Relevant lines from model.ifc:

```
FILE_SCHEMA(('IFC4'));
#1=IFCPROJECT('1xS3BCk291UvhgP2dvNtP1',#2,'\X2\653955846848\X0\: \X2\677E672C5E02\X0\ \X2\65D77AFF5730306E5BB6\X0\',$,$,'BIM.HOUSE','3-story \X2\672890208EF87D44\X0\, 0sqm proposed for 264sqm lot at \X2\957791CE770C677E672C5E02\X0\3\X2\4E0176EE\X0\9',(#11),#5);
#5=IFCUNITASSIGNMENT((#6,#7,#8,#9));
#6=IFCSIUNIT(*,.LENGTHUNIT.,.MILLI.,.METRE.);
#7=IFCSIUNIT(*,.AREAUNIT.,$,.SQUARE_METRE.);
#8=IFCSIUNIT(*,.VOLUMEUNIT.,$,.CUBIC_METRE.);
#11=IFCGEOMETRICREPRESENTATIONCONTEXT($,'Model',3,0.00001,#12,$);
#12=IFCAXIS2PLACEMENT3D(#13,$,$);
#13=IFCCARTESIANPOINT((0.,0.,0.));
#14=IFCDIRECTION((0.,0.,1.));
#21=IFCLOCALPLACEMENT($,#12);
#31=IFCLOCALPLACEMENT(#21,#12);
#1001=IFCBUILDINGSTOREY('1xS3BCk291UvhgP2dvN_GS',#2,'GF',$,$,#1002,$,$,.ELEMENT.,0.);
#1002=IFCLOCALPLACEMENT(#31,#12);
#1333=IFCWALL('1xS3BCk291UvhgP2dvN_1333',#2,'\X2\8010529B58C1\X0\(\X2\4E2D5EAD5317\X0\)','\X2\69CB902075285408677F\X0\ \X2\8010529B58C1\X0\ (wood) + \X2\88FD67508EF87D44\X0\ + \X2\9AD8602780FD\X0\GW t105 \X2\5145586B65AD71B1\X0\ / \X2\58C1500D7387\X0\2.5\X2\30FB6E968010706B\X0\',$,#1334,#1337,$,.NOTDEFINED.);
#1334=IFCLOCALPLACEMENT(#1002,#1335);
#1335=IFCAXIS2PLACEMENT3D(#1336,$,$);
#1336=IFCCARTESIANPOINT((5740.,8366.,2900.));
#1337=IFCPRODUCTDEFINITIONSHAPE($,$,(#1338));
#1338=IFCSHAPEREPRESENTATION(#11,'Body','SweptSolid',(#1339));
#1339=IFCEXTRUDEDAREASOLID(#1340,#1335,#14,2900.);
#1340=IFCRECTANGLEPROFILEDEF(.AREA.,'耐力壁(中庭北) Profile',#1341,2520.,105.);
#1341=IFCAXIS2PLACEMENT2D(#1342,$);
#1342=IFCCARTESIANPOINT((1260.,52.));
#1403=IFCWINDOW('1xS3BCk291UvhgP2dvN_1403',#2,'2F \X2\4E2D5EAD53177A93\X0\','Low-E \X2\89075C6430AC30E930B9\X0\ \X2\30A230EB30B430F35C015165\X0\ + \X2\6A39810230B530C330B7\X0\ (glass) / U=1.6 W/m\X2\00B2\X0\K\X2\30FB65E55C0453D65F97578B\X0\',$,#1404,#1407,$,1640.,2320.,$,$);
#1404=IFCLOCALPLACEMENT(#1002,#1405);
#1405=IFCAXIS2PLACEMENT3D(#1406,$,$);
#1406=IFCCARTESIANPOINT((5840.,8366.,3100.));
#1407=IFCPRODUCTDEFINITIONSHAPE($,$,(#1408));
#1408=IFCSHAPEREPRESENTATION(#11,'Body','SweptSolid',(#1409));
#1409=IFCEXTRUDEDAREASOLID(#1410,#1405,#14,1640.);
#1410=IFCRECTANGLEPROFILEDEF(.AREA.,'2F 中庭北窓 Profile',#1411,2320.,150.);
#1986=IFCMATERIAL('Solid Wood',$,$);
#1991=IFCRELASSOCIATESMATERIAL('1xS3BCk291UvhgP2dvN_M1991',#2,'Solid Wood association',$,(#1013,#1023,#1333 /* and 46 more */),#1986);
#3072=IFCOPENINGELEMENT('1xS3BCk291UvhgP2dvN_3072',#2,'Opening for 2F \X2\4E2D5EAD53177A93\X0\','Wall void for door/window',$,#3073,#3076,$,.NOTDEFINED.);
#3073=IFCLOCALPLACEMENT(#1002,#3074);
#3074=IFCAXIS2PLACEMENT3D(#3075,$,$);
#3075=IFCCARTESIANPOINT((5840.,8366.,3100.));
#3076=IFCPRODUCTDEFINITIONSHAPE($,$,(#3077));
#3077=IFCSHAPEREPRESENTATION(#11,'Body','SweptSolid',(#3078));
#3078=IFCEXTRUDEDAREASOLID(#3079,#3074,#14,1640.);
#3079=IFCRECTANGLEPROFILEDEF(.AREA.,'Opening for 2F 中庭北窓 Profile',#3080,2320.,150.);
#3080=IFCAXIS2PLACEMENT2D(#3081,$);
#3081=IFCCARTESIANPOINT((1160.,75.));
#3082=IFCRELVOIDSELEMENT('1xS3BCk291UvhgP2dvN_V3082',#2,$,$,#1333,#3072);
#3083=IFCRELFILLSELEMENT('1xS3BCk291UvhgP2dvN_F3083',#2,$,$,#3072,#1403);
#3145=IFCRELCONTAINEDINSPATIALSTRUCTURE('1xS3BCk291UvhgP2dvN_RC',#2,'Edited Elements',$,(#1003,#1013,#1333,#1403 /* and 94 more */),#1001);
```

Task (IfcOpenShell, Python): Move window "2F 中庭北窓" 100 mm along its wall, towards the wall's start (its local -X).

```python
import ifcopenshell
import ifcopenshell.api.geometry
import ifcopenshell.util.placement
import ifcopenshell.util.unit

model = ifcopenshell.open("model.ifc")
unit_scale = ifcopenshell.util.unit.calculate_unit_scale(model)

window = model.by_id(1403)
opening = window.FillsVoids[0].RelatingOpeningElement
wall = opening.VoidsElements[0].RelatingBuildingElement

wall_matrix = ifcopenshell.util.placement.get_local_placement(wall.ObjectPlacement)
shift = wall_matrix[:3, 0] * -0.1 / unit_scale
before = ifcopenshell.util.placement.get_local_placement(window.ObjectPlacement)[:3, 3].copy()

# The window is not placed relative to its opening, so move both.
for product in (opening, window):
    matrix = ifcopenshell.util.placement.get_local_placement(product.ObjectPlacement)
    matrix[:3, 3] += shift
    ifcopenshell.api.geometry.edit_object_placement(model, product=product, matrix=matrix, is_si=False)

after = ifcopenshell.util.placement.get_local_placement(window.ObjectPlacement)[:3, 3]
print("window moved by", (after - before).round(3) + 0.0)

model.write("model_updated.ifc")
```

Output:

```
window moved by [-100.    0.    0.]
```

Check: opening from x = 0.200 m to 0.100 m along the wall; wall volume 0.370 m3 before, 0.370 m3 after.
